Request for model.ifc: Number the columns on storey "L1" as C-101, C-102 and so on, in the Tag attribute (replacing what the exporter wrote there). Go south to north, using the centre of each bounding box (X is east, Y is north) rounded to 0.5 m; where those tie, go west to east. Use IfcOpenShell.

First a look at what the model holds.

```python
import ifcopenshell
import ifcopenshell.util.element
import ifcopenshell.util.placement

model = ifcopenshell.open("model.ifc")
print(model.schema)
storey = next(s for s in model.by_type("IfcBuildingStorey") if s.Name == "L1")
columns = [e for e in ifcopenshell.util.element.get_decomposition(storey) if e.is_a("IfcColumn")]
for e in sorted(columns, key=lambda e: e.id()):
    origin = ifcopenshell.util.placement.get_local_placement(e.ObjectPlacement)[:3, 3]
    print(e.id(), e.Tag, e.Name, origin.round(2) + 0.0, sep=" | ")
```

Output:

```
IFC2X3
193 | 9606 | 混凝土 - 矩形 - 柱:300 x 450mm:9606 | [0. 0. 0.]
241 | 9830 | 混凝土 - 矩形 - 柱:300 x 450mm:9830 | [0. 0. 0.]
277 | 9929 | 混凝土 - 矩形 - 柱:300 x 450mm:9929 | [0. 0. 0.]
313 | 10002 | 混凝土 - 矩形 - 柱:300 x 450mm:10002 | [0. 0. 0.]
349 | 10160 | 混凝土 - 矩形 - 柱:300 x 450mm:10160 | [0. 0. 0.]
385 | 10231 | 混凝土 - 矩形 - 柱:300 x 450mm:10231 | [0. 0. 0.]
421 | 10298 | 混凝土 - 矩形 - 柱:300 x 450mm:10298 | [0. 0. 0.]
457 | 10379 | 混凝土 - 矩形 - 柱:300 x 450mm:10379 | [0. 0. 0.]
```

```python
import ifcopenshell
import ifcopenshell.geom
import ifcopenshell.util.element
import ifcopenshell.util.shape

model = ifcopenshell.open("model.ifc")
settings = ifcopenshell.geom.settings()
settings.set("use-world-coords", True)


def centre(element):
    shape = ifcopenshell.geom.create_shape(settings, element)
    return ifcopenshell.util.shape.get_bbox_centroid(shape.geometry)


storey = next(s for s in model.by_type("IfcBuildingStorey") if s.Name == "L1")
columns = [e for e in ifcopenshell.util.element.get_decomposition(storey) if e.is_a("IfcColumn")]

# Insertion points can sit at a corner or the storey origin, so sort by the geometry (in metres).
centres = {e: centre(e) for e in columns}
columns.sort(key=lambda e: (round(centres[e][1] / 0.5), centres[e][0]))

for i, e in enumerate(columns, start=1):
    number = f"C-1{i:02d}"
    e.Tag = number
    print(e.id(), number)

model.write("model_updated.ifc")
```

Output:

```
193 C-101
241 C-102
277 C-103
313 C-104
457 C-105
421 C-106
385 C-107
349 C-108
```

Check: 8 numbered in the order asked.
